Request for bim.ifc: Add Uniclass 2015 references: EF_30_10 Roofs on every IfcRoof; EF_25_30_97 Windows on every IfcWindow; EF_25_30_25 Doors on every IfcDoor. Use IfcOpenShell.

First a look at what the model holds.

```python
import ifcopenshell

model = ifcopenshell.open("bim.ifc")
print(model.schema)
print("classifications:", [c.Name for c in model.by_type("IfcClassification")])
for ifc_class in ("IfcDoor", "IfcRoof", "IfcStair", "IfcWall", "IfcWindow"):
    print(ifc_class, len(model.by_type(ifc_class)))
```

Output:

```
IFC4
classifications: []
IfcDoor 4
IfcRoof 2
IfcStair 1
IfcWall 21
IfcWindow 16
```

```python
import ifcopenshell
import ifcopenshell.api.classification

model = ifcopenshell.open("bim.ifc")

system = ifcopenshell.api.classification.add_classification(model, classification="Uniclass 2015")

codes = {
    "IfcRoof": ("EF_30_10", "Roofs"),
    "IfcWindow": ("EF_25_30_97", "Windows"),
    "IfcDoor": ("EF_25_30_25", "Doors"),
}
for ifc_class, (code, name) in codes.items():
    products = model.by_type(ifc_class)
    ifcopenshell.api.classification.add_reference(
        model, products=products, classification=system, identification=code, name=name
    )
    print(code, len(products))

model.write("bim_updated.ifc")
```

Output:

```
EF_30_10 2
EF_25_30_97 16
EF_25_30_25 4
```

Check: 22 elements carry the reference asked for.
